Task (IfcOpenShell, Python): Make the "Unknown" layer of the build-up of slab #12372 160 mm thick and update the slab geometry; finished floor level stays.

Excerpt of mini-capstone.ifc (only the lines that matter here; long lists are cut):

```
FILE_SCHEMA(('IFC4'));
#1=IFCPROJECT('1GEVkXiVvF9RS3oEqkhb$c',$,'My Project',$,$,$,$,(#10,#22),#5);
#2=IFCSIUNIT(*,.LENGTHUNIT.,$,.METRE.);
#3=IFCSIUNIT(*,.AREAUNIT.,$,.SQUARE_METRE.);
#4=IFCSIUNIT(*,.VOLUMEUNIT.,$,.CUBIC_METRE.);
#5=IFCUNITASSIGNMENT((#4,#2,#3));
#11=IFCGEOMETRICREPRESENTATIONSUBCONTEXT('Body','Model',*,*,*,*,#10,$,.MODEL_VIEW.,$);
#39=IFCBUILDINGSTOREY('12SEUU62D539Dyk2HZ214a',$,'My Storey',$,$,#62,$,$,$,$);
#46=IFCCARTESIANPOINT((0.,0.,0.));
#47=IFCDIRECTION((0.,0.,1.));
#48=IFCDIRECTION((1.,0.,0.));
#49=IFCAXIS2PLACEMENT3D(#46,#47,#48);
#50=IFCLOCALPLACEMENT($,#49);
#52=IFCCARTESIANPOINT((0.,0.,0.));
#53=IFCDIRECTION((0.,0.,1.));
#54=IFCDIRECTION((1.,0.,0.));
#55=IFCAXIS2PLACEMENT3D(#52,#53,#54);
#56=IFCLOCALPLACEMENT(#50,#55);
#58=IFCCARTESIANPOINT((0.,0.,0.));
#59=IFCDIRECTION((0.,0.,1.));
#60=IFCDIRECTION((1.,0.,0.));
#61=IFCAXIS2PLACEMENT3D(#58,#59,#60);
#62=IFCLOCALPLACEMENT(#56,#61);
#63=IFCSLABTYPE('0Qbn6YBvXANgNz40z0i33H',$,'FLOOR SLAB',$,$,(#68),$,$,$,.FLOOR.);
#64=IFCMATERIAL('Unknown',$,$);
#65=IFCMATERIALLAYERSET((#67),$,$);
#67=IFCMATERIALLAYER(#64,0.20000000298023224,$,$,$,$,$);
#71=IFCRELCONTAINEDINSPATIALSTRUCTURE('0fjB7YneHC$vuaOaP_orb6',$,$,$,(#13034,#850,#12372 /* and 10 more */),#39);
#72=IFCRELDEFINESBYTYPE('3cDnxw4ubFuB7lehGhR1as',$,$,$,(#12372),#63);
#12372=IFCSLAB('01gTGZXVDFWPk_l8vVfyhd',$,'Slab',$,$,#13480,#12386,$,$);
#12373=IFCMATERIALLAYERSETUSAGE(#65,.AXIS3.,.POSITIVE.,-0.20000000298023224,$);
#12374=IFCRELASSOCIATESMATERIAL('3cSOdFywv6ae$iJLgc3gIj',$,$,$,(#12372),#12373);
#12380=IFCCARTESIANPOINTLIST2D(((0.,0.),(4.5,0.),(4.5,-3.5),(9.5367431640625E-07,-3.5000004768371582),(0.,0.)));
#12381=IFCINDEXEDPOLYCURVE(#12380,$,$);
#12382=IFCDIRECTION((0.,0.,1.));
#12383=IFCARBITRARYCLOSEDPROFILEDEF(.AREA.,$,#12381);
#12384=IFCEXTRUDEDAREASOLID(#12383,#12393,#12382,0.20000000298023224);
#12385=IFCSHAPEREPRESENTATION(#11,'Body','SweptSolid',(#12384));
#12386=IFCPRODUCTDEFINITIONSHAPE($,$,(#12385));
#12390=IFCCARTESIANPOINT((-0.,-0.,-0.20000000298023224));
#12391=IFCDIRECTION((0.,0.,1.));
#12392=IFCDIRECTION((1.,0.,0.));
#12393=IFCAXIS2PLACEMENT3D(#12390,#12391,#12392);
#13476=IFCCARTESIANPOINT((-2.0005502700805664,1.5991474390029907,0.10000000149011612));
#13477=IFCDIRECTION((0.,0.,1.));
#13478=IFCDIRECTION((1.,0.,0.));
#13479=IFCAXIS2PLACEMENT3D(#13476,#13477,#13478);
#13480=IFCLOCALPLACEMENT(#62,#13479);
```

```python
import ifcopenshell
import ifcopenshell.util.element
import ifcopenshell.util.representation

model = ifcopenshell.open("mini-capstone.ifc")

layer_set = model.by_id(65)
layer = next(l for l in layer_set.MaterialLayers if l.Material and l.Material.Name == "Unknown")
change = 0.16 - layer.LayerThickness
layer.LayerThickness += change

# Geometry does not follow the layer set by itself.
slabs = [e for e in ifcopenshell.util.element.get_elements_by_material(model, layer_set) if e.is_a("IfcSlab")]
for slab in sorted(slabs, key=lambda e: e.id()):
    body = ifcopenshell.util.representation.get_representation(slab, "Model", "Body")
    solid = body.Items[0]
    old_depth = solid.Depth
    solid.Depth += change
    # Extruded upwards: lower the start of the extrusion so the top stays.
    x, y, z = solid.Position.Location.Coordinates
    solid.Position.Location = model.createIfcCartesianPoint((x, y, z - change))
    print(slab.id(), f"{old_depth:g} -> {solid.Depth:g}")

# The layers are counted up from the underside, which has moved.
for usage in {ifcopenshell.util.element.get_material(slab) for slab in slabs}:
    usage.OffsetFromReferenceLine -= change

model.write("mini-capstone_rev.ifc")
```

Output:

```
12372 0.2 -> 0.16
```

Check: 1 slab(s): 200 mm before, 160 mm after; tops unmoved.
